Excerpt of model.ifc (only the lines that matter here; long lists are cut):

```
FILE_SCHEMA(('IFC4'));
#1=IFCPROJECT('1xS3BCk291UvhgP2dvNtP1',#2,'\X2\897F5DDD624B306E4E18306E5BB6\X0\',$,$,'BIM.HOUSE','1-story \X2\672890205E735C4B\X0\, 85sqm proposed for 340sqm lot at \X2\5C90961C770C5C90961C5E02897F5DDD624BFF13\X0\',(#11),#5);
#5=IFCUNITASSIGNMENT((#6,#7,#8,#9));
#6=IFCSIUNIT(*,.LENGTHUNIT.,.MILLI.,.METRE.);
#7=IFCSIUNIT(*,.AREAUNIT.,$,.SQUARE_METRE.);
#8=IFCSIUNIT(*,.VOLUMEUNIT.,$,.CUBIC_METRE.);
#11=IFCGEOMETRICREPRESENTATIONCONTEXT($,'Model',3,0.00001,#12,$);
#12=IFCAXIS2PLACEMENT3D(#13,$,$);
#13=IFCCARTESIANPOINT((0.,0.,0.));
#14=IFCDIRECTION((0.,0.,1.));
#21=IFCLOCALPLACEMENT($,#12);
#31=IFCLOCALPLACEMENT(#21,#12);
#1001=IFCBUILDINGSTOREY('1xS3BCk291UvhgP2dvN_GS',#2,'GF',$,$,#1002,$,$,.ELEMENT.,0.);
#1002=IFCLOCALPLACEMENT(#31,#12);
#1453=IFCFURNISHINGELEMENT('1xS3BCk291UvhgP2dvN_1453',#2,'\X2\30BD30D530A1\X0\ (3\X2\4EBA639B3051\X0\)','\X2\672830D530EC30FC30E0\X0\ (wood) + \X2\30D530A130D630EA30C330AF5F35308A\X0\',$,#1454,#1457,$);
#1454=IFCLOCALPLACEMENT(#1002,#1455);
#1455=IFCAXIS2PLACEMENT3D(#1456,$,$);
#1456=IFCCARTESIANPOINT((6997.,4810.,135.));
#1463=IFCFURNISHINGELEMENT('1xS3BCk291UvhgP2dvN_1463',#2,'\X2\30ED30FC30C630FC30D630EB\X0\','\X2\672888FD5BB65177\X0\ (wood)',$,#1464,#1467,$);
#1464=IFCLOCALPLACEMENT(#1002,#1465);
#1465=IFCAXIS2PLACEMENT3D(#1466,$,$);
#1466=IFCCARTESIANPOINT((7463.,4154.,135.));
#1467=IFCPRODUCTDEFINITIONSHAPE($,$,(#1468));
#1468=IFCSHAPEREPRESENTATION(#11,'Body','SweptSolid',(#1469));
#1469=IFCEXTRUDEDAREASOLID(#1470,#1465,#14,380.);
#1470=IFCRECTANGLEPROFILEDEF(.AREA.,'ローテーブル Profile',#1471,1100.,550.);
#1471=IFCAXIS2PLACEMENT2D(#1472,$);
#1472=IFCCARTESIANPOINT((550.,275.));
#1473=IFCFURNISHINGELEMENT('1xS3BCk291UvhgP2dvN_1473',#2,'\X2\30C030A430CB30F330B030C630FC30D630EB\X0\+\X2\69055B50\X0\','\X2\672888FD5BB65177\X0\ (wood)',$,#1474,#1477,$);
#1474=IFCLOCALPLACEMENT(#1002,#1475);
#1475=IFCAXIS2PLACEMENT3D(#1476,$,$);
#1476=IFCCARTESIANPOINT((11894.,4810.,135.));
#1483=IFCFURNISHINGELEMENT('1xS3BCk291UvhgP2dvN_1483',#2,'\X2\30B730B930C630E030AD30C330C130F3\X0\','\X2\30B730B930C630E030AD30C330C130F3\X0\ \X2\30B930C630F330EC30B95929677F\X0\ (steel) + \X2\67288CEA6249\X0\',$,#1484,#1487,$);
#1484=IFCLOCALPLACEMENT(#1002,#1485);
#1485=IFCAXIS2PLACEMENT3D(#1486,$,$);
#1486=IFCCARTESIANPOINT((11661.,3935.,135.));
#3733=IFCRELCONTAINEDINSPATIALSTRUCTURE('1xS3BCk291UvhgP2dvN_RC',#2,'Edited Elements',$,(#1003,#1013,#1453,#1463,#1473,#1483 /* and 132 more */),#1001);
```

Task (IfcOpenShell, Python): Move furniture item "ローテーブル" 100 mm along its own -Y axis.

```python
import ifcopenshell
import ifcopenshell.api.geometry
import ifcopenshell.util.placement
import ifcopenshell.util.unit

model = ifcopenshell.open("model.ifc")
unit_scale = ifcopenshell.util.unit.calculate_unit_scale(model)

item = model.by_guid("1xS3BCk291UvhgP2dvN_1463")
matrix = ifcopenshell.util.placement.get_local_placement(item.ObjectPlacement)
matrix[:3, 3] -= matrix[:3, 1] * 0.1 / unit_scale
ifcopenshell.api.geometry.edit_object_placement(model, product=item, matrix=matrix, is_si=False)

print(ifcopenshell.util.placement.get_local_placement(item.ObjectPlacement).round(3) + 0.0)

model.write("model_rev.ifc")
```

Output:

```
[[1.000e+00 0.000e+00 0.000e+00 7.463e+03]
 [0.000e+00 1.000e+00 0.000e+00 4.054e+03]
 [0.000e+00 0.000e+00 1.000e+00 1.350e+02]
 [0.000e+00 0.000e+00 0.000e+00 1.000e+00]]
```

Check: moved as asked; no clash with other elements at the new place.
